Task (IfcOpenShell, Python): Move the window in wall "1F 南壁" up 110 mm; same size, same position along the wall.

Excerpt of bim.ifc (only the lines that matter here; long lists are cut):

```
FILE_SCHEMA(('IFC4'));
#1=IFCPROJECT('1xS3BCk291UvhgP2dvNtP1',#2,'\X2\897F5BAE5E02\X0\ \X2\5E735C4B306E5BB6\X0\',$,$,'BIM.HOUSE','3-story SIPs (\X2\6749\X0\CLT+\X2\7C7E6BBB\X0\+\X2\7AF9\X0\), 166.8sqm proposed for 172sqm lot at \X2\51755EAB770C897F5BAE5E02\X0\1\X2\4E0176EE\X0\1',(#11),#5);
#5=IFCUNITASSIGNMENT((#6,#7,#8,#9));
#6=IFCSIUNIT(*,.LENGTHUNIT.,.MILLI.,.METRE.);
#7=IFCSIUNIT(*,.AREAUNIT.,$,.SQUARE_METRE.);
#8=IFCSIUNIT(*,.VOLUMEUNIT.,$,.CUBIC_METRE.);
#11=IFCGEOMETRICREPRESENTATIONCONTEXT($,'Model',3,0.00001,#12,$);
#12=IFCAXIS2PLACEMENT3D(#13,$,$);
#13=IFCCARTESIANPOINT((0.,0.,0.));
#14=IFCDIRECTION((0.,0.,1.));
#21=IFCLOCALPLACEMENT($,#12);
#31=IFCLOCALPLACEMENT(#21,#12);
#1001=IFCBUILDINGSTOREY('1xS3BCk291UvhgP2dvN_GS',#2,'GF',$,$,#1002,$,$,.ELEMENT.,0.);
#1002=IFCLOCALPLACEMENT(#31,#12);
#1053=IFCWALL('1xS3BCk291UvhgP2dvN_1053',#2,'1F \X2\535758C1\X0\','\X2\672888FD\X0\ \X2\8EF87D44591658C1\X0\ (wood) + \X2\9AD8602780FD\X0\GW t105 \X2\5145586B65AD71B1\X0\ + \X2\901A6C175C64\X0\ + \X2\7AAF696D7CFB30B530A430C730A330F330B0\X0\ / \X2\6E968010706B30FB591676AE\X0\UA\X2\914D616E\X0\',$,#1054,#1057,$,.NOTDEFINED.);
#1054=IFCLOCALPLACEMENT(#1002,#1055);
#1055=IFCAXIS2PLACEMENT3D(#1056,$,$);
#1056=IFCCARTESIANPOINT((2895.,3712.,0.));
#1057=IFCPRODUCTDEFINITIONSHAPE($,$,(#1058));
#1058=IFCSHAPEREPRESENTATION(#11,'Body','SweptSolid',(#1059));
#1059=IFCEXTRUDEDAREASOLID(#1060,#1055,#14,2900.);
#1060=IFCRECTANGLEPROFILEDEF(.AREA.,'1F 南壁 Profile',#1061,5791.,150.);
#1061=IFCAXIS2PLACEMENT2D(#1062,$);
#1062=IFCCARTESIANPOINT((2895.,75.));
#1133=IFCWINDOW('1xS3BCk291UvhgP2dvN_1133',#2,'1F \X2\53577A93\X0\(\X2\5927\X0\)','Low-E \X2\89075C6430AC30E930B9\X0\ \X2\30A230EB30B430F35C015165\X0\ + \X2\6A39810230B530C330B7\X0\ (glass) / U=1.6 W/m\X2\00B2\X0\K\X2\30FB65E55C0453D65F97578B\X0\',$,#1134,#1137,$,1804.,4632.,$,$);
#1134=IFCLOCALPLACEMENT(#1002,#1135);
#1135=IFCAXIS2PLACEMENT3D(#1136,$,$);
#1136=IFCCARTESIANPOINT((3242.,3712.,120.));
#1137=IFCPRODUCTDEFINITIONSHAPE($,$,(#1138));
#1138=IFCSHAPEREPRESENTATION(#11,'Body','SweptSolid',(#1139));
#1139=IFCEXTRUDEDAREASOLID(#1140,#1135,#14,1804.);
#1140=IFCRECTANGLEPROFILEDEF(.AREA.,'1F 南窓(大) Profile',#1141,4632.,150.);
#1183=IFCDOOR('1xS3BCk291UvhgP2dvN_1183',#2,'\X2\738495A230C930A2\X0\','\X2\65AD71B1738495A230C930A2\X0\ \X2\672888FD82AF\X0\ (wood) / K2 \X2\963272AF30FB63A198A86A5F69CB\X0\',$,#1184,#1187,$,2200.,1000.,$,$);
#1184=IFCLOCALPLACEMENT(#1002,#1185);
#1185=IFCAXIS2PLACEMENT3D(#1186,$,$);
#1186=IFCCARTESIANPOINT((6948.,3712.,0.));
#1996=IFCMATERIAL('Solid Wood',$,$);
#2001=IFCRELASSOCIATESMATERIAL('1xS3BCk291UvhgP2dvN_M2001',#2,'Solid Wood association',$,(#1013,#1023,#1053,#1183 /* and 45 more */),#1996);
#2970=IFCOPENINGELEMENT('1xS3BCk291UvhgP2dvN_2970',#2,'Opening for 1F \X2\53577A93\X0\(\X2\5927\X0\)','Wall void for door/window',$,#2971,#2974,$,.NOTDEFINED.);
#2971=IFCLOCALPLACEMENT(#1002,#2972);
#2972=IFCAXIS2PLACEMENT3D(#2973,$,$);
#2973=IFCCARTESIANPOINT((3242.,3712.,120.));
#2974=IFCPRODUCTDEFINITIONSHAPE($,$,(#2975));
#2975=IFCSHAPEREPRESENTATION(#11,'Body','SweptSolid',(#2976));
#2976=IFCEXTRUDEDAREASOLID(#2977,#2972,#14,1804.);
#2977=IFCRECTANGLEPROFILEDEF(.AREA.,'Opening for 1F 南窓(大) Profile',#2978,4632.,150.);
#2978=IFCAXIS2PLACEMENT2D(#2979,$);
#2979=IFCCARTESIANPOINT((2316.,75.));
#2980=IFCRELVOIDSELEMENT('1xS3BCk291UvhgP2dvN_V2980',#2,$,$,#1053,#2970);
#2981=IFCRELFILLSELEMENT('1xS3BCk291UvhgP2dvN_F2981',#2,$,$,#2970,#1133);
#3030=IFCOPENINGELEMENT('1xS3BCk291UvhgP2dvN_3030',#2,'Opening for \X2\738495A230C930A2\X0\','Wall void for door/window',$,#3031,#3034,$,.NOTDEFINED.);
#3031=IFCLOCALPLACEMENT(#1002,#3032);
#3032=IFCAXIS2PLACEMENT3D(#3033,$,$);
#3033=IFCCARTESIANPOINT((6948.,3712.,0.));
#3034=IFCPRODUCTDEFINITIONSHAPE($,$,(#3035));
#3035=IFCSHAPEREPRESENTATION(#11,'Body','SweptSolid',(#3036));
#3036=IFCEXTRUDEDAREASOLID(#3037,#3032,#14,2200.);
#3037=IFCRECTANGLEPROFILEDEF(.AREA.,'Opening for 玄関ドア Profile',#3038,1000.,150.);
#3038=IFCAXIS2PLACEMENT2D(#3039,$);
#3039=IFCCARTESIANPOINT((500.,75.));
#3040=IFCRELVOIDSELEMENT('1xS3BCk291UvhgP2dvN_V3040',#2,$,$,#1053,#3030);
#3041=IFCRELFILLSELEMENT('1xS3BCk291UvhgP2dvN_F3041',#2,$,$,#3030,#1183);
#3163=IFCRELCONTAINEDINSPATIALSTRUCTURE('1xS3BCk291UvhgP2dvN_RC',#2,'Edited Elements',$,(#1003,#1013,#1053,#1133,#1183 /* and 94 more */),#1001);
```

```python
import numpy as np
import ifcopenshell
import ifcopenshell.api.geometry
import ifcopenshell.util.placement
import ifcopenshell.util.unit

model = ifcopenshell.open("bim.ifc")
unit_scale = ifcopenshell.util.unit.calculate_unit_scale(model)

window = model.by_id(1133)
opening = window.FillsVoids[0].RelatingOpeningElement
dz = 110.0

shift = np.array([0.0, 0.0, dz])
# The window is not placed relative to its opening, so move both.
for product in (opening, window):
    matrix = ifcopenshell.util.placement.get_local_placement(product.ObjectPlacement)
    matrix[:3, 3] += shift
    ifcopenshell.api.geometry.edit_object_placement(model, product=product, matrix=matrix, is_si=False)

print(f"moved by {dz * unit_scale:+.3f} m")

model.write("bim_v2.ifc")
```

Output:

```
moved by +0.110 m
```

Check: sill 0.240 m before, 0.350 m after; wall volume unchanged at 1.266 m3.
